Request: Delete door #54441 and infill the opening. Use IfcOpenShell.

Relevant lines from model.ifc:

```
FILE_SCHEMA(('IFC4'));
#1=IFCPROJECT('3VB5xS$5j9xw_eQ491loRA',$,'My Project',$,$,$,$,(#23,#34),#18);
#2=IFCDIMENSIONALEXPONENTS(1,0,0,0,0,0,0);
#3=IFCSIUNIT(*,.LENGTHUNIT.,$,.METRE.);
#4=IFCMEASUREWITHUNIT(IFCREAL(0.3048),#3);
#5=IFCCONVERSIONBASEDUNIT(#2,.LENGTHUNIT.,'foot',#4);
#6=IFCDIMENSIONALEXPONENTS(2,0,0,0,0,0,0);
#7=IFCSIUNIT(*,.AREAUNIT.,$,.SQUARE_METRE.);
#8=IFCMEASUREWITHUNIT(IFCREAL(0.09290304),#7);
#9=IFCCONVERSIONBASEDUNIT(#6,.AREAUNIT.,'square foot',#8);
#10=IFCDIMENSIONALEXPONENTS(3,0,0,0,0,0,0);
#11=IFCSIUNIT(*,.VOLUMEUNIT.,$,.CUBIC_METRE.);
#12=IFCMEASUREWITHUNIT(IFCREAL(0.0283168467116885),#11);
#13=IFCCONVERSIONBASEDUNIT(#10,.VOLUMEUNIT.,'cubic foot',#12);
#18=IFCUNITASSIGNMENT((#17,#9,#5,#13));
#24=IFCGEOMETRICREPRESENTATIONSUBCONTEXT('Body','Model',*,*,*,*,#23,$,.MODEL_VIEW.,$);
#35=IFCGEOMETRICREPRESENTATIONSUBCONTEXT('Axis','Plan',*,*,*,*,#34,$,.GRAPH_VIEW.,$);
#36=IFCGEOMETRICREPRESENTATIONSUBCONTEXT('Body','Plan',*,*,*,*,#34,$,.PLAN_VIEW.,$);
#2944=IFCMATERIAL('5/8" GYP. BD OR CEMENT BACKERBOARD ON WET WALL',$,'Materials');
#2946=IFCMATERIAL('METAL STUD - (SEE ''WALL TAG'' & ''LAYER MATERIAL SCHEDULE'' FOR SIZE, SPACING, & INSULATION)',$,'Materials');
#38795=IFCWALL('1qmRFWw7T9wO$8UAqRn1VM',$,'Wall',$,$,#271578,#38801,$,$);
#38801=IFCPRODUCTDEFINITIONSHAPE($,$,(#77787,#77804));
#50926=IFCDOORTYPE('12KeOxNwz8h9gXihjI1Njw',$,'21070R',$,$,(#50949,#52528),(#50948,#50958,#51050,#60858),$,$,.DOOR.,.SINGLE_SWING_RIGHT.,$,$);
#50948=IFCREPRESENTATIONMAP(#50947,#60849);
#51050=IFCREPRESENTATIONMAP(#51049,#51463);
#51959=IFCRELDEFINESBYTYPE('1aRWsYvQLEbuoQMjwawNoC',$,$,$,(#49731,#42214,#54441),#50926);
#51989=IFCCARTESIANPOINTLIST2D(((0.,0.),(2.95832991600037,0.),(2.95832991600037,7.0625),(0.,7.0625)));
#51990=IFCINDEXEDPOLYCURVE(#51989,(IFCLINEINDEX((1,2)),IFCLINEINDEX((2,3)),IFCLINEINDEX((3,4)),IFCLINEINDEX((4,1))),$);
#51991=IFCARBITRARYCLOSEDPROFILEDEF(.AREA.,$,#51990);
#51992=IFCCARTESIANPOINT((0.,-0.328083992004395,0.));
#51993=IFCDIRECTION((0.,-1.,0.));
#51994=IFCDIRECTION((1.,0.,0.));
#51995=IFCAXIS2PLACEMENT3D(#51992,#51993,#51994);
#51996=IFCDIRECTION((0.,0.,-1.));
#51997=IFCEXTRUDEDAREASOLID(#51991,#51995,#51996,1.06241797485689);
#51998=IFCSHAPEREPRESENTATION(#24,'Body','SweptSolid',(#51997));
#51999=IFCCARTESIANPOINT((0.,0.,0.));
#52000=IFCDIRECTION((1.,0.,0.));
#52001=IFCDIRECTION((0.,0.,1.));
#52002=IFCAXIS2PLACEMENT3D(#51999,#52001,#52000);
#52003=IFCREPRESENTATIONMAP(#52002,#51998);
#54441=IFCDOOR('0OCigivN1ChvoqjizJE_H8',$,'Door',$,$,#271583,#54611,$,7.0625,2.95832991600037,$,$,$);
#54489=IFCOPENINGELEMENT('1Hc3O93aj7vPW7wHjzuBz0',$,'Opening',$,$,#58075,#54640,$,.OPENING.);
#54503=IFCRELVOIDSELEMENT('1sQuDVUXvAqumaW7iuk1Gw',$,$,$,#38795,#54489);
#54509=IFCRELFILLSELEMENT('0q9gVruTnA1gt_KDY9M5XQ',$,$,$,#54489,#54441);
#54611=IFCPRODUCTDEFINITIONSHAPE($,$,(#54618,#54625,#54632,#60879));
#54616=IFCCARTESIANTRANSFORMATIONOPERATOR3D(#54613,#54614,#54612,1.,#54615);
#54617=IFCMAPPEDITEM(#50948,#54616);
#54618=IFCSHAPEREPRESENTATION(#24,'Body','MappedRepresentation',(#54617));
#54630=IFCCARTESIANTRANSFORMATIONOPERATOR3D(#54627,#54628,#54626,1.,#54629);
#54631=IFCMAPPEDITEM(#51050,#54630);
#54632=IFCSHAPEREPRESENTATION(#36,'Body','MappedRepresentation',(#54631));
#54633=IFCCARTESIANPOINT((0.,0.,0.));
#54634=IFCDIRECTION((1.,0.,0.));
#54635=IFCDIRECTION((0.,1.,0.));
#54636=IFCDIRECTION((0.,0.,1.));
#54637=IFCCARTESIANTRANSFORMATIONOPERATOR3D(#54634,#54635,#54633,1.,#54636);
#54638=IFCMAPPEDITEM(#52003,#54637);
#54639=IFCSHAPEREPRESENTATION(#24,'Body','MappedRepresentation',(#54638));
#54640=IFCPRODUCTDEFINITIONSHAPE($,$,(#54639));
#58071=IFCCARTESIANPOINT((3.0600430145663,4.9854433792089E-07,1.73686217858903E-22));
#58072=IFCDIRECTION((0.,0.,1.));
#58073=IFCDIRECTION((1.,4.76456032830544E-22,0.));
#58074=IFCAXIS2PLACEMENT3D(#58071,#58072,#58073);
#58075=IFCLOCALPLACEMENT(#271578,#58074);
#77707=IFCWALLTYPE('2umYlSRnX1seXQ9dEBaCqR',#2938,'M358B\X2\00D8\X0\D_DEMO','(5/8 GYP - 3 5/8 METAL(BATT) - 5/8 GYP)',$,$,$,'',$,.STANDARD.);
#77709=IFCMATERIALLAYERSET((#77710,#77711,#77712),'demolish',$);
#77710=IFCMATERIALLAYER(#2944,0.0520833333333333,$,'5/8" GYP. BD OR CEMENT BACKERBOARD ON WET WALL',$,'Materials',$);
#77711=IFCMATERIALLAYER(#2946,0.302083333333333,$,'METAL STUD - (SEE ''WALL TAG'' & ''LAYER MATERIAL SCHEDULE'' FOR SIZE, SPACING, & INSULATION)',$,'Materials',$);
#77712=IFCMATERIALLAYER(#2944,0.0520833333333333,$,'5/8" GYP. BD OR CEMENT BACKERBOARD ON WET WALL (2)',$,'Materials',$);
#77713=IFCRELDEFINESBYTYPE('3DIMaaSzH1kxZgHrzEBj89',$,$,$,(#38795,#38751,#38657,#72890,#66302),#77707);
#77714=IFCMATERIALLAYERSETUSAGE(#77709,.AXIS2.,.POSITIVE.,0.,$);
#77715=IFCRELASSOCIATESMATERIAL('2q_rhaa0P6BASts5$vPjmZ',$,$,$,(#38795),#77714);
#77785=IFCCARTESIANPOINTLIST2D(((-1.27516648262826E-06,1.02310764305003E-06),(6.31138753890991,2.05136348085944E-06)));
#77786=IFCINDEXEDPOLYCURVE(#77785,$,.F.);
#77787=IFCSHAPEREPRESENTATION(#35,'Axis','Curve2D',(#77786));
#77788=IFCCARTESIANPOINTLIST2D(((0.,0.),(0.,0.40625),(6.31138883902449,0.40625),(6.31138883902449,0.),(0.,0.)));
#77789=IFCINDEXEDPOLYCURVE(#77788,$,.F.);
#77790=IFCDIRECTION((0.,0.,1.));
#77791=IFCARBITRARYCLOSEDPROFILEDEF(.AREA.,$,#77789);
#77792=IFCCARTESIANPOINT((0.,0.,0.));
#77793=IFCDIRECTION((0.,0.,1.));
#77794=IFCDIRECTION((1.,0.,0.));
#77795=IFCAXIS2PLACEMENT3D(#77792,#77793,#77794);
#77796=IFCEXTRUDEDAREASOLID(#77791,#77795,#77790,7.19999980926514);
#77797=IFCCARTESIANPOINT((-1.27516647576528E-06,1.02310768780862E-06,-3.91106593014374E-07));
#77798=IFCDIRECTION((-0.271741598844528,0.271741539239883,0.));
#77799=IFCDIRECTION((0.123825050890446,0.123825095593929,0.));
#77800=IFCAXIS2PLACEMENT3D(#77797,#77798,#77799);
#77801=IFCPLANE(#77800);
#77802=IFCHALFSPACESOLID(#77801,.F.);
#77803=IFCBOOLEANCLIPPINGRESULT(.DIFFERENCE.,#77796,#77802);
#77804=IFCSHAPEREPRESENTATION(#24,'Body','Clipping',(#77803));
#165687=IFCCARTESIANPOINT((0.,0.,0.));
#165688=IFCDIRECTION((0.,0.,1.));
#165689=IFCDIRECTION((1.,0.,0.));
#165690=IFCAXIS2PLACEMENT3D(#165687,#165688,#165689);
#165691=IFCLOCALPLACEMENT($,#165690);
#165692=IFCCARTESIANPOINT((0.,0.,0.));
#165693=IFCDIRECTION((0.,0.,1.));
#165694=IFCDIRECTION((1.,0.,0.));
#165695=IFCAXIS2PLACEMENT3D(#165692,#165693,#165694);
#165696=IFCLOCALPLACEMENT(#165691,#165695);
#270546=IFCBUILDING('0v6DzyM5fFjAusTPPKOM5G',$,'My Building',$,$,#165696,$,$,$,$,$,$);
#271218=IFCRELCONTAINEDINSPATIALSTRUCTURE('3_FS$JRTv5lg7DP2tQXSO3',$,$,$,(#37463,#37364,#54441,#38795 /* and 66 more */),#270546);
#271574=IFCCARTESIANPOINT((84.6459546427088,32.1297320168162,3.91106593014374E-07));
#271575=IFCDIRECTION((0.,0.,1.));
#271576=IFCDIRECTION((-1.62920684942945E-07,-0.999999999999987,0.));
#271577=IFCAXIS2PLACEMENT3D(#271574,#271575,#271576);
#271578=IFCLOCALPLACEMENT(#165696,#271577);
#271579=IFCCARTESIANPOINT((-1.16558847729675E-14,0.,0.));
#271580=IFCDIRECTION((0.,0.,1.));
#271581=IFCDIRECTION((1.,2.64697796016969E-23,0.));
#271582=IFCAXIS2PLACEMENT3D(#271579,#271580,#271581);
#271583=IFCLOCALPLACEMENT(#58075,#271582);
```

```python
import ifcopenshell
import ifcopenshell.api.feature
import ifcopenshell.api.root
import ifcopenshell.geom
import ifcopenshell.util.shape

model = ifcopenshell.open("model.ifc")
settings = ifcopenshell.geom.settings()


def volume(element):
    """Net volume in cubic metres, openings subtracted."""
    shape = ifcopenshell.geom.create_shape(settings, element)
    return ifcopenshell.util.shape.get_volume(shape.geometry)


door = model.by_guid("0OCigivN1ChvoqjizJE_H8")
opening = door.FillsVoids[0].RelatingOpeningElement
wall = opening.VoidsElements[0].RelatingBuildingElement
before = volume(wall)

ifcopenshell.api.root.remove_product(model, product=door)
ifcopenshell.api.feature.remove_feature(model, feature=opening)

after = volume(wall)

print(f"wall volume {before:.3f} -> {after:.3f} m3")

model.write("model_edited.ifc")
```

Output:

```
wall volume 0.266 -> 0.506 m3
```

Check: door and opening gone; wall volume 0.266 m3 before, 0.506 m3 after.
